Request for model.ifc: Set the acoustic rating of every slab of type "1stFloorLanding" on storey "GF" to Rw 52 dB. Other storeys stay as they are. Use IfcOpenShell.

First a look at what the model holds.

```python
import ifcopenshell
import ifcopenshell.util.element

model = ifcopenshell.open("model.ifc")
print(model.schema)
storey = next(s for s in model.by_type("IfcBuildingStorey") if s.Name == "GF")
slabs = [e for e in ifcopenshell.util.element.get_decomposition(storey) if e.is_a("IfcSlab")]
seen = {}
for e in slabs:
    element_type = ifcopenshell.util.element.get_type(e)
    key = (element_type.Name if element_type != e and element_type else None, ifcopenshell.util.element.get_pset(e, "Pset_SlabCommon", "AcousticRating"))
    seen[key] = seen.get(key, 0) + 1
for (name, value), count in sorted(seen.items(), key=str):
    print(count, "x", name, "|", value)
```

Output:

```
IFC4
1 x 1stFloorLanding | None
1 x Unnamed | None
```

```python
import ifcopenshell
import ifcopenshell.api.pset
import ifcopenshell.util.element

model = ifcopenshell.open("model.ifc")

storey = next(s for s in model.by_type("IfcBuildingStorey") if s.Name == "GF")
slabs = [e for e in ifcopenshell.util.element.get_decomposition(storey) if e.is_a("IfcSlab")]

count = 0
for e in slabs:
    element_type = ifcopenshell.util.element.get_type(e)
    if element_type in (None, e) or element_type.Name != "1stFloorLanding":
        continue
    # add_pset returns the element's existing set when there is one.
    pset = ifcopenshell.api.pset.add_pset(model, product=e, name="Pset_SlabCommon")
    ifcopenshell.api.pset.edit_pset(model, pset=pset, properties={"AcousticRating": "Rw 52 dB"})
    count += 1

print(count, "slabs updated")

model.write("model_rev.ifc")
```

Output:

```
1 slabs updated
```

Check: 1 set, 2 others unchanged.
